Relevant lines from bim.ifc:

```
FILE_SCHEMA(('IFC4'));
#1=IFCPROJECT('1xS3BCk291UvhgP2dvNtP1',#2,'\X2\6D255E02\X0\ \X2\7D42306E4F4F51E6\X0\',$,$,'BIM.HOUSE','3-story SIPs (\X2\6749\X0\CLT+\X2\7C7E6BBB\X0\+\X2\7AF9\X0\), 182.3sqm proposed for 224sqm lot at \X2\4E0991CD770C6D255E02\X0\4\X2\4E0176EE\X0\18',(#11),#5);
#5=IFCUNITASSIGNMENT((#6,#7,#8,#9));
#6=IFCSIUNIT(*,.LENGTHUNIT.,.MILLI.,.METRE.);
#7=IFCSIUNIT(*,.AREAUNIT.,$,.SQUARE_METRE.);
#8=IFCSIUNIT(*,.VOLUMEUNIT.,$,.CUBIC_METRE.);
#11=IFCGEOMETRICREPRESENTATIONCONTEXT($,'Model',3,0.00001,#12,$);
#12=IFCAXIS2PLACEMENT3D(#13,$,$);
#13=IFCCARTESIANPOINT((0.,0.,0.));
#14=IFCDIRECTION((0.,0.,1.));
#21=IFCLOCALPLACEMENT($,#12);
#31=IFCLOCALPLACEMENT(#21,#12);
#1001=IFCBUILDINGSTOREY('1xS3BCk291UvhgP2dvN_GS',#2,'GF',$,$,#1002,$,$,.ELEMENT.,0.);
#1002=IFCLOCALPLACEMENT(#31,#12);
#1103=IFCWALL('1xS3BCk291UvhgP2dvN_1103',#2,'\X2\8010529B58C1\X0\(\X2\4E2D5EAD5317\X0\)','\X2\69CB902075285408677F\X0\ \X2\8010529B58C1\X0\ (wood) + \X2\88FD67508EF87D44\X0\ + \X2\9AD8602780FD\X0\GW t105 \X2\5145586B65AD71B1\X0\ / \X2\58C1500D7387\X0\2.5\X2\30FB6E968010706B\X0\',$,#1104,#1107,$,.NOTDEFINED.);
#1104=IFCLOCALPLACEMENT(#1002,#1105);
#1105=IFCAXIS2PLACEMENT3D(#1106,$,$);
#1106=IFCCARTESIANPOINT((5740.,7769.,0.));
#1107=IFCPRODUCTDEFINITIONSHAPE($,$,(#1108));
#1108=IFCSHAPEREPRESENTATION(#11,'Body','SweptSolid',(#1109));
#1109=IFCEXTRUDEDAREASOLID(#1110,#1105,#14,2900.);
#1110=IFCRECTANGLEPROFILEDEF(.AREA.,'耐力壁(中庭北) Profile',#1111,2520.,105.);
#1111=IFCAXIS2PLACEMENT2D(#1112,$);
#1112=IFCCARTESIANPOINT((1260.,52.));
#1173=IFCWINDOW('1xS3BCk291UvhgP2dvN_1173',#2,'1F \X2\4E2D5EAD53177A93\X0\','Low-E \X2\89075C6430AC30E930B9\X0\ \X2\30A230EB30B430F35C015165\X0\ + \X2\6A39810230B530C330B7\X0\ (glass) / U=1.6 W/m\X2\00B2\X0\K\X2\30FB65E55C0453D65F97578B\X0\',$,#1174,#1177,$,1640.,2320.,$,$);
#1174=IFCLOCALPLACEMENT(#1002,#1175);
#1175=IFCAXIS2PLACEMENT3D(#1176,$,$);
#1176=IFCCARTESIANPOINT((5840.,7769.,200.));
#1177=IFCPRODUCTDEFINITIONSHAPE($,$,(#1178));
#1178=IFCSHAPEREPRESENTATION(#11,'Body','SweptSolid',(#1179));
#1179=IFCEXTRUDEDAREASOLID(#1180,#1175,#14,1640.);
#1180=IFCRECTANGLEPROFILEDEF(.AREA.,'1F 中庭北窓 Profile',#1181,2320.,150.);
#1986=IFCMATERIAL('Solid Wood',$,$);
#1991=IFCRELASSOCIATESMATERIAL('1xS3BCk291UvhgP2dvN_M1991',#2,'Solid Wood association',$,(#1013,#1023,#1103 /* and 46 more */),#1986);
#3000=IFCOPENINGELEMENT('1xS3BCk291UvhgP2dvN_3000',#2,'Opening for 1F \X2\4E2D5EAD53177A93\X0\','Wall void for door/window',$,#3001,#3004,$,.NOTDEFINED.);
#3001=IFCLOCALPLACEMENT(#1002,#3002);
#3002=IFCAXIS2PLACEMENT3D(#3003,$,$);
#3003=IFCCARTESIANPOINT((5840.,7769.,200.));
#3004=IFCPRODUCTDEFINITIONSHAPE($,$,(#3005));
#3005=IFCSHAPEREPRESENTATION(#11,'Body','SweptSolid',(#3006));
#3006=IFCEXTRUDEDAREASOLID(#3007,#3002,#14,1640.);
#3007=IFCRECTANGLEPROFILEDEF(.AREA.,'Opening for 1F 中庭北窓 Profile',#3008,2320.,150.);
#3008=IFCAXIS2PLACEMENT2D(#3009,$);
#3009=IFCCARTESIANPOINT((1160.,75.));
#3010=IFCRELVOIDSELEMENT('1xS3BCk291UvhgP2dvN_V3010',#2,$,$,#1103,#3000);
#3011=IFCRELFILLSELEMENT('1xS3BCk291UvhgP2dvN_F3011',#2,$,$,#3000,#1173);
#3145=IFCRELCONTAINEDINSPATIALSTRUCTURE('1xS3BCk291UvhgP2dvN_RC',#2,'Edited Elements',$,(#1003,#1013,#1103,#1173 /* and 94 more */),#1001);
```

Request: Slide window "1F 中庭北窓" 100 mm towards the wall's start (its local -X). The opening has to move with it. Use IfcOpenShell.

```python
import ifcopenshell
import ifcopenshell.api.geometry
import ifcopenshell.util.placement

model = ifcopenshell.open("bim.ifc")

window = model.by_id(1173)
opening = window.FillsVoids[0].RelatingOpeningElement
wall = opening.VoidsElements[0].RelatingBuildingElement

wall_matrix = ifcopenshell.util.placement.get_local_placement(wall.ObjectPlacement)
shift = wall_matrix[:3, 0] * -100.0
before = ifcopenshell.util.placement.get_local_placement(window.ObjectPlacement)[:3, 3].copy()

# The window is not placed relative to its opening, so move both.
for product in (opening, window):
    matrix = ifcopenshell.util.placement.get_local_placement(product.ObjectPlacement)
    matrix[:3, 3] += shift
    ifcopenshell.api.geometry.edit_object_placement(model, product=product, matrix=matrix, is_si=False)

after = ifcopenshell.util.placement.get_local_placement(window.ObjectPlacement)[:3, 3]
print("window moved by", (after - before).round(3) + 0.0)

model.write("bim_updated.ifc")
```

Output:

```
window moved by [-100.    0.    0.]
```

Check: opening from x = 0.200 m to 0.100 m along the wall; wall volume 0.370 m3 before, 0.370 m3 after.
